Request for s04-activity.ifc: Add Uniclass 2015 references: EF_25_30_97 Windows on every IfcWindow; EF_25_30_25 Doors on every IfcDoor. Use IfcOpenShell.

First a look at what the model holds.

```python
import ifcopenshell

model = ifcopenshell.open("s04-activity.ifc")
print(model.schema)
print("classifications:", [c.Name for c in model.by_type("IfcClassification")])
for ifc_class in ("IfcDoor", "IfcRoof", "IfcStair", "IfcWall", "IfcWindow"):
    print(ifc_class, len(model.by_type(ifc_class)))
```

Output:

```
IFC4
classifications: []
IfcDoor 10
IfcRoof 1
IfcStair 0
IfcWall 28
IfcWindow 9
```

```python
import ifcopenshell
import ifcopenshell.api.classification

model = ifcopenshell.open("s04-activity.ifc")

system = ifcopenshell.api.classification.add_classification(model, classification="Uniclass 2015")

codes = {
    "IfcWindow": ("EF_25_30_97", "Windows"),
    "IfcDoor": ("EF_25_30_25", "Doors"),
}
for ifc_class, (code, name) in codes.items():
    products = model.by_type(ifc_class)
    ifcopenshell.api.classification.add_reference(
        model, products=products, classification=system, identification=code, name=name
    )
    print(code, len(products))

model.write("s04-activity_v2.ifc")
```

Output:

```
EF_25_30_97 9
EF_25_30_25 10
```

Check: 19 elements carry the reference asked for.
